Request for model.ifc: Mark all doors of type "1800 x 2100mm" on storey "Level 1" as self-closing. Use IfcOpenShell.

First a look at what the model holds.

```python
import ifcopenshell
import ifcopenshell.util.element

model = ifcopenshell.open("model.ifc")
print(model.schema)
storey = next(s for s in model.by_type("IfcBuildingStorey") if s.Name == "Level 1")
doors = [e for e in ifcopenshell.util.element.get_decomposition(storey) if e.is_a("IfcDoor")]
seen = {}
for e in doors:
    element_type = ifcopenshell.util.element.get_type(e)
    key = (element_type.Name if element_type != e and element_type else None, ifcopenshell.util.element.get_pset(e, "Pset_DoorCommon", "SelfClosing"))
    seen[key] = seen.get(key, 0) + 1
for (name, value), count in sorted(seen.items(), key=str):
    print(count, "x", name, "|", value)
```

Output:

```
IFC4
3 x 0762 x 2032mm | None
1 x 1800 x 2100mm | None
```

```python
import ifcopenshell
import ifcopenshell.api.pset
import ifcopenshell.util.element

model = ifcopenshell.open("model.ifc")

storey = next(s for s in model.by_type("IfcBuildingStorey") if s.Name == "Level 1")
doors = [e for e in ifcopenshell.util.element.get_decomposition(storey) if e.is_a("IfcDoor")]

count = 0
for e in doors:
    element_type = ifcopenshell.util.element.get_type(e)
    if element_type in (None, e) or element_type.Name != "1800 x 2100mm":
        continue
    # add_pset returns the element's existing set when there is one.
    pset = ifcopenshell.api.pset.add_pset(model, product=e, name="Pset_DoorCommon")
    ifcopenshell.api.pset.edit_pset(model, pset=pset, properties={"SelfClosing": True})
    count += 1

print(count, "doors updated")

model.write("model_rev.ifc")
```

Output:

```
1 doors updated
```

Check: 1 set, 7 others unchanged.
